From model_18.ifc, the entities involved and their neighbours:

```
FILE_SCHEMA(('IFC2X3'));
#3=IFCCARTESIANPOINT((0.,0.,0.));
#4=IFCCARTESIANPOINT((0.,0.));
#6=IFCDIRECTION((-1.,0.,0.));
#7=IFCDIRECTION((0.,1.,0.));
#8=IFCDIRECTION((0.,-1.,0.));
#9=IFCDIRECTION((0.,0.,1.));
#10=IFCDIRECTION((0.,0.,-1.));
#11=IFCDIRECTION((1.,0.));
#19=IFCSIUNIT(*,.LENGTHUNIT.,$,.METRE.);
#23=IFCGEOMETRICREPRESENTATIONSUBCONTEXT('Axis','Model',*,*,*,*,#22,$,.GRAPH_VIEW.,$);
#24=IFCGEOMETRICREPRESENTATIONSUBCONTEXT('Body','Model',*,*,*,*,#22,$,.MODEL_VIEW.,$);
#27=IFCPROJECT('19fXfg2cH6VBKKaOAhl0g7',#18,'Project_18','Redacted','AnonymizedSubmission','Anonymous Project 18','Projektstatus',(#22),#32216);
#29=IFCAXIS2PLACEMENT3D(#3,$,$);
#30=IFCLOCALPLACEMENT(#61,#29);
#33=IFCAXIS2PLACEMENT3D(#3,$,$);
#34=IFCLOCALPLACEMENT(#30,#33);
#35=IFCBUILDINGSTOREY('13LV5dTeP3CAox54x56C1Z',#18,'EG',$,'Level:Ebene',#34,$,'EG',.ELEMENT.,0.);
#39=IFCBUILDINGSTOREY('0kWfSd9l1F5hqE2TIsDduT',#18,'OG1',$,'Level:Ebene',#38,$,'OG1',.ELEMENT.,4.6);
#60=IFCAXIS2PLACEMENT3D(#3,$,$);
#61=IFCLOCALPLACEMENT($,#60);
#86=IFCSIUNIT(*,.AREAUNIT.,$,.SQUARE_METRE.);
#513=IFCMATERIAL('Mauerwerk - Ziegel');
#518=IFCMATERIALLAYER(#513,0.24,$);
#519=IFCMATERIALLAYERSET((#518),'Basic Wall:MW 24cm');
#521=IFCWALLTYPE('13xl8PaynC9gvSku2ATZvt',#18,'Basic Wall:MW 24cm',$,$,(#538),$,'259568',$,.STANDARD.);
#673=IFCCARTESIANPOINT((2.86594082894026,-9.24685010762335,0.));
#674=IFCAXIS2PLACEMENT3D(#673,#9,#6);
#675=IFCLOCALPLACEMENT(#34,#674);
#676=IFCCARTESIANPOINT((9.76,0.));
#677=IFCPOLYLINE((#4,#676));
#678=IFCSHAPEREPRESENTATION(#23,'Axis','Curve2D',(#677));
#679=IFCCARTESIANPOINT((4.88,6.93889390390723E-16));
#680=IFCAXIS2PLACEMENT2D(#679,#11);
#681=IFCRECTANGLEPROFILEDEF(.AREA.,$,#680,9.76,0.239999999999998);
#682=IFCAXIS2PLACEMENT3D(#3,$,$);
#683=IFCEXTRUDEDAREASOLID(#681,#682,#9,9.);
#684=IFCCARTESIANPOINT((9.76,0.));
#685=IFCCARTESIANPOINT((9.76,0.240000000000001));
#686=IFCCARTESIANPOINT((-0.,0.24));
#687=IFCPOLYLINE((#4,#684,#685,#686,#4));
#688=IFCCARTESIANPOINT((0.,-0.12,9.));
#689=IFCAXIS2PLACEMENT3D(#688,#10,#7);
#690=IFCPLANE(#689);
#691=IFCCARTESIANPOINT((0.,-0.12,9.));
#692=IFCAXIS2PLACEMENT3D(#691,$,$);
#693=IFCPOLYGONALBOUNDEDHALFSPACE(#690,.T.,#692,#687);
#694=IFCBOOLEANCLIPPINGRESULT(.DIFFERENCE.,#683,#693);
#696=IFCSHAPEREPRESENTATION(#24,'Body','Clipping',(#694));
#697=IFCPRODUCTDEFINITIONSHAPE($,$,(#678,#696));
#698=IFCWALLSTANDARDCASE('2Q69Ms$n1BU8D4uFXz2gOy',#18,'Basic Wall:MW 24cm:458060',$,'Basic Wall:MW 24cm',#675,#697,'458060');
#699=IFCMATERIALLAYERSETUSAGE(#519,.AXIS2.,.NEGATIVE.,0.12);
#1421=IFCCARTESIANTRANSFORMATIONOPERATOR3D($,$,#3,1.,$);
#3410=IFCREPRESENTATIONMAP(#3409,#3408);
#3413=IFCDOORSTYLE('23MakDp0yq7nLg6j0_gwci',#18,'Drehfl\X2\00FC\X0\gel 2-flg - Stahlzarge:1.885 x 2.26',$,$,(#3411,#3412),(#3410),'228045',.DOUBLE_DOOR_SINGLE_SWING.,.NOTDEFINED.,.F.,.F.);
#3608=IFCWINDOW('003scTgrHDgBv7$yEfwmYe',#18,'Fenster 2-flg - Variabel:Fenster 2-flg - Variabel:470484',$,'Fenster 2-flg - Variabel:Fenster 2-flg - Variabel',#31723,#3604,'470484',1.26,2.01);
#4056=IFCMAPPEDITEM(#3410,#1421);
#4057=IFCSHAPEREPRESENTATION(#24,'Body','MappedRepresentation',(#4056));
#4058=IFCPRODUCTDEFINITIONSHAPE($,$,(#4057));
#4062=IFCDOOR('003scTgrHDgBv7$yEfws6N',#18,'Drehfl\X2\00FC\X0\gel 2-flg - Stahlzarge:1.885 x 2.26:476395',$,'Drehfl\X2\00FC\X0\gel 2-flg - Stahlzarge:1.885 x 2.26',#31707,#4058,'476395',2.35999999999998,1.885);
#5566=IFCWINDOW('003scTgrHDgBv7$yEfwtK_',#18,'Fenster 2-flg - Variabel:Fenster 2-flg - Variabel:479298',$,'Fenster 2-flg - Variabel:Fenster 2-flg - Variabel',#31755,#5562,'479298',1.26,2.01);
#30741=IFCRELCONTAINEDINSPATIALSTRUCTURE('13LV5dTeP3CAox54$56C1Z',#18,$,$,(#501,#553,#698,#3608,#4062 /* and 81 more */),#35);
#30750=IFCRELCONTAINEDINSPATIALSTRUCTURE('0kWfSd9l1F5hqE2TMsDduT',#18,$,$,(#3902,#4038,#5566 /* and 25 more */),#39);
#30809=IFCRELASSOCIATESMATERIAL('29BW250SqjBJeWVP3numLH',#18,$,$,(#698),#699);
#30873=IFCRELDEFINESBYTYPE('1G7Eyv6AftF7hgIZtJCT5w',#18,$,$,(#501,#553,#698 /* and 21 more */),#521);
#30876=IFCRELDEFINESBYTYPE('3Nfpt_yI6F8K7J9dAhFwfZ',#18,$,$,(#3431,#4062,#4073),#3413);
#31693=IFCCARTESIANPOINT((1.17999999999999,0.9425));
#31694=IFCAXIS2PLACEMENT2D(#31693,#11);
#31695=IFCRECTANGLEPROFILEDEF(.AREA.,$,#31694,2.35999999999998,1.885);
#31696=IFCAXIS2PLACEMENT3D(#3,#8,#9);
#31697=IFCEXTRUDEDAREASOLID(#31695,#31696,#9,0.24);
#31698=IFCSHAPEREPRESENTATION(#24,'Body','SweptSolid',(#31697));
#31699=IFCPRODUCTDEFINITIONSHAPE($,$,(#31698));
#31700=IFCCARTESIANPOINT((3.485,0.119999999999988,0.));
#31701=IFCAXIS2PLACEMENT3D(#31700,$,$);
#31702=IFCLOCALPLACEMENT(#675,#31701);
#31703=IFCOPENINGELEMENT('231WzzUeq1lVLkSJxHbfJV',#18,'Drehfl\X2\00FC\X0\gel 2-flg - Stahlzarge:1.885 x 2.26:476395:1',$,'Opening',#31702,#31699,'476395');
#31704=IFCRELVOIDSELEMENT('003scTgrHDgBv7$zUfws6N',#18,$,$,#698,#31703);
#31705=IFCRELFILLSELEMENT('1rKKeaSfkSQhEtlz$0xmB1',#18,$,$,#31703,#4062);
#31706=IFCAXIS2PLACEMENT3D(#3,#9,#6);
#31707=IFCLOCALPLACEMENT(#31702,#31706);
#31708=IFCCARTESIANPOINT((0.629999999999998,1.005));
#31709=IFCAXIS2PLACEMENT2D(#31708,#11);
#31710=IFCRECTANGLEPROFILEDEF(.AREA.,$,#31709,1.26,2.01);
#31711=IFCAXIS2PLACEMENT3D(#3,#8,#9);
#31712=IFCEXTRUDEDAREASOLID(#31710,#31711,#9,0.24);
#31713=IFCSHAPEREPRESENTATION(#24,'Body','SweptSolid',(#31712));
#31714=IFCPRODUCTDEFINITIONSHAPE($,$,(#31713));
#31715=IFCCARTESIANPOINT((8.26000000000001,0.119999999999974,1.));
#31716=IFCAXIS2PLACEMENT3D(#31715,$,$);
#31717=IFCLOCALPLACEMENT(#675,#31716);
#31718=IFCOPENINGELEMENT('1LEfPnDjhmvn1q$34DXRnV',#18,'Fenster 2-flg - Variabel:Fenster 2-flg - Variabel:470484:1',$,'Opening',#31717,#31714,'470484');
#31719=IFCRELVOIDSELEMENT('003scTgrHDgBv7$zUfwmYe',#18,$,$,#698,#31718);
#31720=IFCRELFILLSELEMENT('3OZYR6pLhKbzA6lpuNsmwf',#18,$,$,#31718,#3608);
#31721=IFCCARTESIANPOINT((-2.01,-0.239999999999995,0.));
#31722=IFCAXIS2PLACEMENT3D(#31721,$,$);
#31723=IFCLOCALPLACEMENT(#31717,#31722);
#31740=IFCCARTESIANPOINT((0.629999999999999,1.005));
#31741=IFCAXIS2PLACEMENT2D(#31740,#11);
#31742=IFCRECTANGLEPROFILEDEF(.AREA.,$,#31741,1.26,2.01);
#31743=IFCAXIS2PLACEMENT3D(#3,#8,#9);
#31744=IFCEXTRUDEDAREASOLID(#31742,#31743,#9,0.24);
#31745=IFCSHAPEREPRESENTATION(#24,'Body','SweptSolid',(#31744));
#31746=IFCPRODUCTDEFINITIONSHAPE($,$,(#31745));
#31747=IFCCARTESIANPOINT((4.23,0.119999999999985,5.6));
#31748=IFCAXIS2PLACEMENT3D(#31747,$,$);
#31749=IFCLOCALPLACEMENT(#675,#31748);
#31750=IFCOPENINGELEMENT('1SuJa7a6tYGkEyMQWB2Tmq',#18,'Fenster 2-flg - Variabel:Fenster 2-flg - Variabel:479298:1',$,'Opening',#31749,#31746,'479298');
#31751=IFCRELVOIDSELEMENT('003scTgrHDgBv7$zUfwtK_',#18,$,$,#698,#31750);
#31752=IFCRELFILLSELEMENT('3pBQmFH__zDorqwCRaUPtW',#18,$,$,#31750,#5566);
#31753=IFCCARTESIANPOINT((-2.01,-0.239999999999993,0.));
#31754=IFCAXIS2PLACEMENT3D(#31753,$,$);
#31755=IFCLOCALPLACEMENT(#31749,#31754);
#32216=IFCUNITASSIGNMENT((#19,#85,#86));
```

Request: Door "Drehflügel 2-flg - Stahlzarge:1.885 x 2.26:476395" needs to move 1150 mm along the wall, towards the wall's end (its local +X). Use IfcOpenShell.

```python
import ifcopenshell
import ifcopenshell.api.geometry
import ifcopenshell.util.placement

model = ifcopenshell.open("model_18.ifc")

door = model.by_guid("003scTgrHDgBv7$yEfws6N")
opening = door.FillsVoids[0].RelatingOpeningElement
wall = opening.VoidsElements[0].RelatingBuildingElement

wall_matrix = ifcopenshell.util.placement.get_local_placement(wall.ObjectPlacement)
shift = wall_matrix[:3, 0] * 1.15
before = ifcopenshell.util.placement.get_local_placement(door.ObjectPlacement)[:3, 3].copy()

# The door is placed relative to its opening, so it follows when the opening moves.
matrix = ifcopenshell.util.placement.get_local_placement(opening.ObjectPlacement)
matrix[:3, 3] += shift
ifcopenshell.api.geometry.edit_object_placement(
    model, product=opening, matrix=matrix, is_si=False, should_transform_children=True
)

after = ifcopenshell.util.placement.get_local_placement(door.ObjectPlacement)[:3, 3]
print("door moved by", (after - before).round(3) + 0.0)

model.write("model_18_v2.ifc")
```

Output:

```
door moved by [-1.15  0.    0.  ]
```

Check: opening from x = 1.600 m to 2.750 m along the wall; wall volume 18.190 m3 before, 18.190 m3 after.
